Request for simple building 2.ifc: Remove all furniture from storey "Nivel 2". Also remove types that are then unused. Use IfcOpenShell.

First a look at what the model holds.

```python
import ifcopenshell
import ifcopenshell.util.element

model = ifcopenshell.open("simple building 2.ifc")
print(model.schema)
storey = next(s for s in model.by_type("IfcBuildingStorey") if s.Name == "Nivel 2")
furniture = [e for e in ifcopenshell.util.element.get_decomposition(storey) if e.is_a("IfcFurnishingElement")]
seen = {}
for e in furniture:
    element_type = ifcopenshell.util.element.get_type(e)
    name = element_type.Name if element_type not in (None, e) else None
    seen[name] = seen.get(name, 0) + 1
for name, count in sorted(seen.items(), key=str):
    print(count, "x", name)
```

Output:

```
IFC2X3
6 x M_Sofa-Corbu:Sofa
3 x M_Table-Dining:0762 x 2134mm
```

```python
import ifcopenshell
import ifcopenshell.api.root
import ifcopenshell.util.element

model = ifcopenshell.open("simple building 2.ifc")

storey = next(s for s in model.by_type("IfcBuildingStorey") if s.Name == "Nivel 2")
furniture = [e for e in ifcopenshell.util.element.get_decomposition(storey) if e.is_a("IfcFurnishingElement")]
types = {ifcopenshell.util.element.get_type(e) for e in furniture} - {None, *furniture}

for e in furniture:
    ifcopenshell.api.root.remove_product(model, product=e)
print(len(furniture), "removed")

unused = [t for t in types if not ifcopenshell.util.element.get_types(t)]
for t in unused:
    ifcopenshell.api.root.remove_product(model, product=t)
print(len(unused), "unused types removed")

model.write("simple building 2-out.ifc")
```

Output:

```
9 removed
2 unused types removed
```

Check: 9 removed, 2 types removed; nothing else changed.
